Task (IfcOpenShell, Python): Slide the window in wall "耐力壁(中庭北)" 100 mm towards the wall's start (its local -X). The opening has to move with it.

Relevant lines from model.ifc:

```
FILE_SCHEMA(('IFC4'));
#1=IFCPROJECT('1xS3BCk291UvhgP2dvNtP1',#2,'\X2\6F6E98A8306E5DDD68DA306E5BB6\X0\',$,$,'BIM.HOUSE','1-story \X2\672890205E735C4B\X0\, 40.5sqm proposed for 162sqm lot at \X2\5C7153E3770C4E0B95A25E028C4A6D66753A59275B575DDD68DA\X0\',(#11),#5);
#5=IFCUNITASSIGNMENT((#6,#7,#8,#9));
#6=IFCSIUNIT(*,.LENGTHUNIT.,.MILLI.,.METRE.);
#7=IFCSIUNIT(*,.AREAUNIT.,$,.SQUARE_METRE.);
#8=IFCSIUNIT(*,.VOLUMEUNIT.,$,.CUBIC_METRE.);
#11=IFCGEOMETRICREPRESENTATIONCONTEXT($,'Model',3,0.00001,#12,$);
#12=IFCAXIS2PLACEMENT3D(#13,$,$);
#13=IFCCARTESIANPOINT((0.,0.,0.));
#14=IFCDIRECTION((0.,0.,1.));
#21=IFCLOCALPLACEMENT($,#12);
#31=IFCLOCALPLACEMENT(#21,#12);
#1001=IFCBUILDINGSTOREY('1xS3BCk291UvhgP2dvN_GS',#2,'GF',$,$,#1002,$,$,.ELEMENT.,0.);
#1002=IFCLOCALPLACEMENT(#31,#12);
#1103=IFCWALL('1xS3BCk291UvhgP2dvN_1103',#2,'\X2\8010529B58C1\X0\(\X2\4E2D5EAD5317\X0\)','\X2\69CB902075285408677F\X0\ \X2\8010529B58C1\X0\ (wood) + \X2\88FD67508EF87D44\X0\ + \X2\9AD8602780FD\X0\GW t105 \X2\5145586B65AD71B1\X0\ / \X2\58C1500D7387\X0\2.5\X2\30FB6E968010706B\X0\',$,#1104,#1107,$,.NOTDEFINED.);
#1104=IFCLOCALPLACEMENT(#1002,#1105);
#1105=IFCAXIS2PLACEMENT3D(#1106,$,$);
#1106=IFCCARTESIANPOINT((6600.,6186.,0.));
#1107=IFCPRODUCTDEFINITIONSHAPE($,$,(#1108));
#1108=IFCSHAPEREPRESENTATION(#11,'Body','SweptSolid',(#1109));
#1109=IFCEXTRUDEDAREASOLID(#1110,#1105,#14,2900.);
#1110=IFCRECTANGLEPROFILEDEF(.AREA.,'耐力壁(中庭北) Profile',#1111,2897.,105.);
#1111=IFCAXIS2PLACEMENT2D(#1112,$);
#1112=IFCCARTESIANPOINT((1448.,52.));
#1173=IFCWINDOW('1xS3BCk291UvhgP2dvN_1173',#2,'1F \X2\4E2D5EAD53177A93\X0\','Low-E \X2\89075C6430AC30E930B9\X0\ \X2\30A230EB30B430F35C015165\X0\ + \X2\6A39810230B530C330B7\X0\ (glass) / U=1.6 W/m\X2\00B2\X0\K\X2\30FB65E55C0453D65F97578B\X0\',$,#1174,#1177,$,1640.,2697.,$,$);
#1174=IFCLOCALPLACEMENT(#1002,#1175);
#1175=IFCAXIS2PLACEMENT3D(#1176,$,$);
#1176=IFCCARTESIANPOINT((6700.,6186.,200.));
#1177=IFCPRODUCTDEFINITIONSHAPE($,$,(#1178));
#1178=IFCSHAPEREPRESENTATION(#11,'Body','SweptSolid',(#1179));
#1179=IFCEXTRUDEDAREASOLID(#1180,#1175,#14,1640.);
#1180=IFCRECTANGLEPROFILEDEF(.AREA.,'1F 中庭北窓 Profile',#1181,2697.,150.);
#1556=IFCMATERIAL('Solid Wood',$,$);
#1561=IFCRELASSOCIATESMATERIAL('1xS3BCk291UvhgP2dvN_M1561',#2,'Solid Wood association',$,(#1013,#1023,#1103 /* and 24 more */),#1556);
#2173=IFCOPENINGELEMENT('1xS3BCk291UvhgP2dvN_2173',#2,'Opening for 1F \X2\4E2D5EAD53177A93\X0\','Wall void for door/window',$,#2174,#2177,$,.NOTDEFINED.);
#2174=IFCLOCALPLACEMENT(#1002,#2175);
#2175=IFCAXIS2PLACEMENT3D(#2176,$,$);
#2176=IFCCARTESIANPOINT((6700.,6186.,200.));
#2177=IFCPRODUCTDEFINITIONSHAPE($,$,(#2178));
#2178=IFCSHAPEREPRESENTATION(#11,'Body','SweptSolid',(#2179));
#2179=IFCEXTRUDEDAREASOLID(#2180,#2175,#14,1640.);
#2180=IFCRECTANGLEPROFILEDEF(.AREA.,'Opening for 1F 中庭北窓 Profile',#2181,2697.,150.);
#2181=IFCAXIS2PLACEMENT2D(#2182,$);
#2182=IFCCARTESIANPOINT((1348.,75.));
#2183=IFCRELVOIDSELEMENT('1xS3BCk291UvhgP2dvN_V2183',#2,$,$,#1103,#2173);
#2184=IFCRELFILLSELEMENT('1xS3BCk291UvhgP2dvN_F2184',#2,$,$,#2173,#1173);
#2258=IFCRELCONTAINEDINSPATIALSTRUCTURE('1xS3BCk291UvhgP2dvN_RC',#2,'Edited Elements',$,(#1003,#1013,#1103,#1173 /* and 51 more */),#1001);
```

```python
import ifcopenshell
import ifcopenshell.api.geometry
import ifcopenshell.util.placement
import ifcopenshell.util.unit

model = ifcopenshell.open("model.ifc")
unit_scale = ifcopenshell.util.unit.calculate_unit_scale(model)

window = model.by_guid("1xS3BCk291UvhgP2dvN_1173")
opening = window.FillsVoids[0].RelatingOpeningElement
wall = opening.VoidsElements[0].RelatingBuildingElement

wall_matrix = ifcopenshell.util.placement.get_local_placement(wall.ObjectPlacement)
shift = wall_matrix[:3, 0] * -0.1 / unit_scale
before = ifcopenshell.util.placement.get_local_placement(window.ObjectPlacement)[:3, 3].copy()

# The window is not placed relative to its opening, so move both.
for product in (opening, window):
    matrix = ifcopenshell.util.placement.get_local_placement(product.ObjectPlacement)
    matrix[:3, 3] += shift
    ifcopenshell.api.geometry.edit_object_placement(model, product=product, matrix=matrix, is_si=False)

after = ifcopenshell.util.placement.get_local_placement(window.ObjectPlacement)[:3, 3]
print("window moved by", (after - before).round(3) + 0.0)

model.write("model_edited.ifc")
```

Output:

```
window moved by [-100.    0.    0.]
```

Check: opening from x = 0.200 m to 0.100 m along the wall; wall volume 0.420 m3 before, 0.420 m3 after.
